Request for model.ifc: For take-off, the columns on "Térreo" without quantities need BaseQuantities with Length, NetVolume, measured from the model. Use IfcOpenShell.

First a look at what the model holds.

```python
import ifcopenshell
import ifcopenshell.util.element
import ifcopenshell.util.unit

model = ifcopenshell.open("model.ifc")
print(model.schema)
for unit_type in ("LENGTHUNIT", "AREAUNIT", "VOLUMEUNIT"):
    print(unit_type, ifcopenshell.util.unit.calculate_unit_scale(model, unit_type))
storey = next(s for s in model.by_type("IfcBuildingStorey") if s.Name == "Térreo")
columns = [e for e in ifcopenshell.util.element.get_decomposition(storey) if e.is_a("IfcColumn")]
for e in sorted(columns, key=lambda e: e.id()):
    print(e.id(), e.is_a(), e.Name, list(ifcopenshell.util.element.get_psets(e, qtos_only=True)), sep=" | ")
```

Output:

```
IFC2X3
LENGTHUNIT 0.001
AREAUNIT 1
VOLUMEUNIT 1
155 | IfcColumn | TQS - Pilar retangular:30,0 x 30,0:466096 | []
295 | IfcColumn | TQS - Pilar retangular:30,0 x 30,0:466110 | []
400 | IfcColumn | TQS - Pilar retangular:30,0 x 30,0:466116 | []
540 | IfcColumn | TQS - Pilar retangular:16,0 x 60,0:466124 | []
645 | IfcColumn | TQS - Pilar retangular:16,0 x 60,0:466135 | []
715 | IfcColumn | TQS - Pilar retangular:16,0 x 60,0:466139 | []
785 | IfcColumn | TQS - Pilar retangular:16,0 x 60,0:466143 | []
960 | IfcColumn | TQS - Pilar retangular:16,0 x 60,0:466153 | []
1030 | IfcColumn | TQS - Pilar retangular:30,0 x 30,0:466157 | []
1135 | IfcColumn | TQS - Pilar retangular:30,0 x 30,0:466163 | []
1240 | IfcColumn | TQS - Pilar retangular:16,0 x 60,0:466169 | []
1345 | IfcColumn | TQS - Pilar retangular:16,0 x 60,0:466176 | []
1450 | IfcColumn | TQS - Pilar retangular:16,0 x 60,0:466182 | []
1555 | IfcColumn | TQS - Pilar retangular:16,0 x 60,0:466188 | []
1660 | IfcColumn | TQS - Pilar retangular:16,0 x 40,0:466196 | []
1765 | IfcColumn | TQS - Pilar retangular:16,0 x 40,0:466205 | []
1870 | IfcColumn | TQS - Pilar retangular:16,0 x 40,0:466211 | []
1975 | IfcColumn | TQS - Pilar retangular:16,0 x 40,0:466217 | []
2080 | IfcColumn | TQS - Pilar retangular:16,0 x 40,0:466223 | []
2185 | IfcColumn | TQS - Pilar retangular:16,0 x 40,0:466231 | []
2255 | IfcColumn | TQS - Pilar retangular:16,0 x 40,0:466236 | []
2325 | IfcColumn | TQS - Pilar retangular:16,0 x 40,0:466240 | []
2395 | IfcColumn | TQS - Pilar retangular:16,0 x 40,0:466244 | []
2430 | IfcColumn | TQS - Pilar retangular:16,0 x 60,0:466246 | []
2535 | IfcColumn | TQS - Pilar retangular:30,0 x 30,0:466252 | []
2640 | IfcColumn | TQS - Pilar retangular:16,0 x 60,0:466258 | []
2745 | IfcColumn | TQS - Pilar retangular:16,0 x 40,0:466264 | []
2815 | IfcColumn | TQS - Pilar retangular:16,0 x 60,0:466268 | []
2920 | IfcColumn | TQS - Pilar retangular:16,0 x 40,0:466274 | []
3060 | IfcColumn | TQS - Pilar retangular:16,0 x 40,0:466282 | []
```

```python
import ifcopenshell
import ifcopenshell.api.pset
import ifcopenshell.geom
import ifcopenshell.util.element
import ifcopenshell.util.shape
import ifcopenshell.util.unit

model = ifcopenshell.open("model.ifc")
unit_scale = ifcopenshell.util.unit.calculate_unit_scale(model)
volume_scale = ifcopenshell.util.unit.calculate_unit_scale(model, "VOLUMEUNIT")
settings = ifcopenshell.geom.settings()

storey = next(s for s in model.by_type("IfcBuildingStorey") if s.Name == "Térreo")
columns = [e for e in ifcopenshell.util.element.get_decomposition(storey) if e.is_a("IfcColumn")]

for e in sorted(columns, key=lambda e: e.id()):
    if ifcopenshell.util.element.get_psets(e, qtos_only=True, should_inherit=False):
        continue
    # Geometry comes back in metres, in the element's own axes.
    shape = ifcopenshell.geom.create_shape(settings, e)
    values = {
        "Length": ifcopenshell.util.shape.get_z(shape.geometry) / unit_scale,
        "NetVolume": ifcopenshell.util.shape.get_volume(shape.geometry) / volume_scale,
    }
    qto = ifcopenshell.api.pset.add_qto(model, product=e, name="BaseQuantities")
    ifcopenshell.api.pset.edit_qto(model, qto=qto, properties=values)
    print(e.id(), {k: round(v, 3) for k, v in values.items()})

model.write("model_updated.ifc")
```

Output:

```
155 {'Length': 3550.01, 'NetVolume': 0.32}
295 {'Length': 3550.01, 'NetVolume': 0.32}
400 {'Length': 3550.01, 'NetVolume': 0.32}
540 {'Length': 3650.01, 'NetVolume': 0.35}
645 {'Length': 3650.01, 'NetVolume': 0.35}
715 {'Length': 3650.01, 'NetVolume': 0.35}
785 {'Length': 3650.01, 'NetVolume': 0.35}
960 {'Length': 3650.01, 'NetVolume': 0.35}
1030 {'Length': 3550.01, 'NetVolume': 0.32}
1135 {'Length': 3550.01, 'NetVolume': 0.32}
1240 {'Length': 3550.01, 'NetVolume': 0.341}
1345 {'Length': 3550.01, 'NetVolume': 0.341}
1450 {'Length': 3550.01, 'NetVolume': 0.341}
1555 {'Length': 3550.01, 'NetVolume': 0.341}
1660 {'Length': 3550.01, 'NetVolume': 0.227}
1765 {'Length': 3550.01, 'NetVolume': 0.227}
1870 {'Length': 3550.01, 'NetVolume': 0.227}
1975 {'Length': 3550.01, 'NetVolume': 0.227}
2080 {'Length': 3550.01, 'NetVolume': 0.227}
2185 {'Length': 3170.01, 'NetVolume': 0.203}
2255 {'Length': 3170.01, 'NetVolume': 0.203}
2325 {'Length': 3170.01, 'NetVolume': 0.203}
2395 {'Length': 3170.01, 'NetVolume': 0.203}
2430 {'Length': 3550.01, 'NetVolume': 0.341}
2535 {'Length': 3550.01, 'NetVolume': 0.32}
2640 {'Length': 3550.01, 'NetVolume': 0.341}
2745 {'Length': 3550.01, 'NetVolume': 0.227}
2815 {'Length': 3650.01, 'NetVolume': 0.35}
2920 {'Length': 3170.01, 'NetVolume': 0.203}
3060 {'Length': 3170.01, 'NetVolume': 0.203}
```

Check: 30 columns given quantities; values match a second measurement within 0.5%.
